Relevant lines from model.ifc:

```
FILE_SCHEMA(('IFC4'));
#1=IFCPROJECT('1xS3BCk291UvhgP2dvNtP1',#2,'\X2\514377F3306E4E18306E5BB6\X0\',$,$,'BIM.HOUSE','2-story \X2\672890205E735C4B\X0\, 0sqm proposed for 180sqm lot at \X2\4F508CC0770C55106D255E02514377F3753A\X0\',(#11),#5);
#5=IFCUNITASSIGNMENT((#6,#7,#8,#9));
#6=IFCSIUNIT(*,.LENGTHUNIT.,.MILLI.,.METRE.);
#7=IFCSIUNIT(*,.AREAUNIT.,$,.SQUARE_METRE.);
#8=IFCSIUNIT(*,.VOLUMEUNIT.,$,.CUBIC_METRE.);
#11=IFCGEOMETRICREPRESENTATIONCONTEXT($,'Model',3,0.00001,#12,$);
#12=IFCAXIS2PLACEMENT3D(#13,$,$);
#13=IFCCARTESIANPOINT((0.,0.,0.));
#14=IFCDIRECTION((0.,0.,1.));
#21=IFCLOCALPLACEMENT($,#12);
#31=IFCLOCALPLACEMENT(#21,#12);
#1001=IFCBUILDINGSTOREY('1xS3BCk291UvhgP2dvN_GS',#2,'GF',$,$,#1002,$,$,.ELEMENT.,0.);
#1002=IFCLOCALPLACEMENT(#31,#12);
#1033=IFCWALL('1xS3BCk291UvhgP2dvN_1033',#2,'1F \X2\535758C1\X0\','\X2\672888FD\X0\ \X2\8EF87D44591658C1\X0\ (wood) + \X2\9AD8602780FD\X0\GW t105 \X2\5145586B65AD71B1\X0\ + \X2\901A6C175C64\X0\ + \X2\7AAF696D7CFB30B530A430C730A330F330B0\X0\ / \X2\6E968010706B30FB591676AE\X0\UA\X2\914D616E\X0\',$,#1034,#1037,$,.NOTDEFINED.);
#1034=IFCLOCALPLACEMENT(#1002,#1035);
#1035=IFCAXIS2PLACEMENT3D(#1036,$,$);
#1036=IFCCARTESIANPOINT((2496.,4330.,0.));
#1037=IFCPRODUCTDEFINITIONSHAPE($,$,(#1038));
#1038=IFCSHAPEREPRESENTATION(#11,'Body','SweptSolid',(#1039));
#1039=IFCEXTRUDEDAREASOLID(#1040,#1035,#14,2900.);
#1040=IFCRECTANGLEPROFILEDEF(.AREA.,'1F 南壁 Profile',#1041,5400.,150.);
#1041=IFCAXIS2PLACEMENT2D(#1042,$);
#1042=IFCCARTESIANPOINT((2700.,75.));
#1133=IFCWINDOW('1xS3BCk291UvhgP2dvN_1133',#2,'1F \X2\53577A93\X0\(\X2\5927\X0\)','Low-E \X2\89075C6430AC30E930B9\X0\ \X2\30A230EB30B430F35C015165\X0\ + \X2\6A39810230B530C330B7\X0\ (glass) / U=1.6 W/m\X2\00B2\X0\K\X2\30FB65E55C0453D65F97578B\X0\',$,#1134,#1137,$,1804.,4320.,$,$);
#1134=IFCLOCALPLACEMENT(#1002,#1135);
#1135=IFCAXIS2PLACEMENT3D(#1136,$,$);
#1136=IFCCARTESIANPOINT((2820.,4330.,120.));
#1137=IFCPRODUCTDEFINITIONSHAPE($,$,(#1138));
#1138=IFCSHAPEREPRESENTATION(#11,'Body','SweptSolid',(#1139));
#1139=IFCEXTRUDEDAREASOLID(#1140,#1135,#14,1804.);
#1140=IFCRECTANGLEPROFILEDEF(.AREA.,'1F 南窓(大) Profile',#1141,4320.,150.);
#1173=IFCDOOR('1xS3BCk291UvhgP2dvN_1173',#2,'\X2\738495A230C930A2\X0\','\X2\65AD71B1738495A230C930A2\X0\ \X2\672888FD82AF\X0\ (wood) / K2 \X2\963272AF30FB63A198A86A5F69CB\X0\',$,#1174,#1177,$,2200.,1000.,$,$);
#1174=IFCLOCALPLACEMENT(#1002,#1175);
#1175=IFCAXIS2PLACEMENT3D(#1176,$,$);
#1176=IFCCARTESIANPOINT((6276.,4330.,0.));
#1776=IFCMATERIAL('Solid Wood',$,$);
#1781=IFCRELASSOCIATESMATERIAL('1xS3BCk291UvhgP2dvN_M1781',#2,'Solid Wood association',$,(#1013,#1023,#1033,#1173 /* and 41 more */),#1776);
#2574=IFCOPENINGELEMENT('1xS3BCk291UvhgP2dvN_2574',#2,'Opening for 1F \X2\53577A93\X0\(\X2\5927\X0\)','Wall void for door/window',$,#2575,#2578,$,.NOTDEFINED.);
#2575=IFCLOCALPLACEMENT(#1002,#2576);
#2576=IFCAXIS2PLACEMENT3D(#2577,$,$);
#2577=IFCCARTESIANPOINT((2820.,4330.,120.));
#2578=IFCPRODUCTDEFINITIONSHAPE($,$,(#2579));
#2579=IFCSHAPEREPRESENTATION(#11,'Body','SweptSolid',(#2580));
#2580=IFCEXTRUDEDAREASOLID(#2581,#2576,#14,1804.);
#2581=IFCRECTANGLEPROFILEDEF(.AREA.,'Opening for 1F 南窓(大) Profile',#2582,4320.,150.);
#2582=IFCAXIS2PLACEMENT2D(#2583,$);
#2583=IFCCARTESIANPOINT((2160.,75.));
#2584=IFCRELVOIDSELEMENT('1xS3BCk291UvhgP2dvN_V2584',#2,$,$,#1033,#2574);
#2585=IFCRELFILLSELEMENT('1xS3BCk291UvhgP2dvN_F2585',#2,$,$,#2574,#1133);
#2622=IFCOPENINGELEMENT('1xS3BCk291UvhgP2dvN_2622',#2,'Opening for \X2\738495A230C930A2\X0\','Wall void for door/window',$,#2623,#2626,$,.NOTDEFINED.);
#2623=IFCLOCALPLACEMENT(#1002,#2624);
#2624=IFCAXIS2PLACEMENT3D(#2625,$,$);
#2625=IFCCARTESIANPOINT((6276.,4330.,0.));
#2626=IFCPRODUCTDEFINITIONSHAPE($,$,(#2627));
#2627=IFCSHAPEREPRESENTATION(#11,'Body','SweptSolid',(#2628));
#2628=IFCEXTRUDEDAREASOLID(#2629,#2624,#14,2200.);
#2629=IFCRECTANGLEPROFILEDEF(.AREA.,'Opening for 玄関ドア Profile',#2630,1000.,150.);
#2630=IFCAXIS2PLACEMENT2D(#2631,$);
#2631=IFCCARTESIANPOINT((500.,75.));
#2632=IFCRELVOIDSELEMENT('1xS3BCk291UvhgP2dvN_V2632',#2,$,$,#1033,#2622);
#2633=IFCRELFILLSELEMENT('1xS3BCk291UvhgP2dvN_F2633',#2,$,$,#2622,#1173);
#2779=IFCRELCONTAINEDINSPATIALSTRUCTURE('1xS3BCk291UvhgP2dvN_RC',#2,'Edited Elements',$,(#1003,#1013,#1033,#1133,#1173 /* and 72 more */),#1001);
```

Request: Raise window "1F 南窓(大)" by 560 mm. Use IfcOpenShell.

```python
import numpy as np
import ifcopenshell
import ifcopenshell.api.geometry
import ifcopenshell.util.placement
import ifcopenshell.util.unit

model = ifcopenshell.open("model.ifc")
unit_scale = ifcopenshell.util.unit.calculate_unit_scale(model)

window = model.by_id(1133)
opening = window.FillsVoids[0].RelatingOpeningElement
dz = 0.56 / unit_scale

shift = np.array([0.0, 0.0, dz])
# The window is not placed relative to its opening, so move both.
for product in (opening, window):
    matrix = ifcopenshell.util.placement.get_local_placement(product.ObjectPlacement)
    matrix[:3, 3] += shift
    ifcopenshell.api.geometry.edit_object_placement(model, product=product, matrix=matrix, is_si=False)

print(f"moved by {dz * unit_scale:+.3f} m")

model.write("model_v2.ifc")
```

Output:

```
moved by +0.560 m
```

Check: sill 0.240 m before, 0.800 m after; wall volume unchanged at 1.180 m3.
